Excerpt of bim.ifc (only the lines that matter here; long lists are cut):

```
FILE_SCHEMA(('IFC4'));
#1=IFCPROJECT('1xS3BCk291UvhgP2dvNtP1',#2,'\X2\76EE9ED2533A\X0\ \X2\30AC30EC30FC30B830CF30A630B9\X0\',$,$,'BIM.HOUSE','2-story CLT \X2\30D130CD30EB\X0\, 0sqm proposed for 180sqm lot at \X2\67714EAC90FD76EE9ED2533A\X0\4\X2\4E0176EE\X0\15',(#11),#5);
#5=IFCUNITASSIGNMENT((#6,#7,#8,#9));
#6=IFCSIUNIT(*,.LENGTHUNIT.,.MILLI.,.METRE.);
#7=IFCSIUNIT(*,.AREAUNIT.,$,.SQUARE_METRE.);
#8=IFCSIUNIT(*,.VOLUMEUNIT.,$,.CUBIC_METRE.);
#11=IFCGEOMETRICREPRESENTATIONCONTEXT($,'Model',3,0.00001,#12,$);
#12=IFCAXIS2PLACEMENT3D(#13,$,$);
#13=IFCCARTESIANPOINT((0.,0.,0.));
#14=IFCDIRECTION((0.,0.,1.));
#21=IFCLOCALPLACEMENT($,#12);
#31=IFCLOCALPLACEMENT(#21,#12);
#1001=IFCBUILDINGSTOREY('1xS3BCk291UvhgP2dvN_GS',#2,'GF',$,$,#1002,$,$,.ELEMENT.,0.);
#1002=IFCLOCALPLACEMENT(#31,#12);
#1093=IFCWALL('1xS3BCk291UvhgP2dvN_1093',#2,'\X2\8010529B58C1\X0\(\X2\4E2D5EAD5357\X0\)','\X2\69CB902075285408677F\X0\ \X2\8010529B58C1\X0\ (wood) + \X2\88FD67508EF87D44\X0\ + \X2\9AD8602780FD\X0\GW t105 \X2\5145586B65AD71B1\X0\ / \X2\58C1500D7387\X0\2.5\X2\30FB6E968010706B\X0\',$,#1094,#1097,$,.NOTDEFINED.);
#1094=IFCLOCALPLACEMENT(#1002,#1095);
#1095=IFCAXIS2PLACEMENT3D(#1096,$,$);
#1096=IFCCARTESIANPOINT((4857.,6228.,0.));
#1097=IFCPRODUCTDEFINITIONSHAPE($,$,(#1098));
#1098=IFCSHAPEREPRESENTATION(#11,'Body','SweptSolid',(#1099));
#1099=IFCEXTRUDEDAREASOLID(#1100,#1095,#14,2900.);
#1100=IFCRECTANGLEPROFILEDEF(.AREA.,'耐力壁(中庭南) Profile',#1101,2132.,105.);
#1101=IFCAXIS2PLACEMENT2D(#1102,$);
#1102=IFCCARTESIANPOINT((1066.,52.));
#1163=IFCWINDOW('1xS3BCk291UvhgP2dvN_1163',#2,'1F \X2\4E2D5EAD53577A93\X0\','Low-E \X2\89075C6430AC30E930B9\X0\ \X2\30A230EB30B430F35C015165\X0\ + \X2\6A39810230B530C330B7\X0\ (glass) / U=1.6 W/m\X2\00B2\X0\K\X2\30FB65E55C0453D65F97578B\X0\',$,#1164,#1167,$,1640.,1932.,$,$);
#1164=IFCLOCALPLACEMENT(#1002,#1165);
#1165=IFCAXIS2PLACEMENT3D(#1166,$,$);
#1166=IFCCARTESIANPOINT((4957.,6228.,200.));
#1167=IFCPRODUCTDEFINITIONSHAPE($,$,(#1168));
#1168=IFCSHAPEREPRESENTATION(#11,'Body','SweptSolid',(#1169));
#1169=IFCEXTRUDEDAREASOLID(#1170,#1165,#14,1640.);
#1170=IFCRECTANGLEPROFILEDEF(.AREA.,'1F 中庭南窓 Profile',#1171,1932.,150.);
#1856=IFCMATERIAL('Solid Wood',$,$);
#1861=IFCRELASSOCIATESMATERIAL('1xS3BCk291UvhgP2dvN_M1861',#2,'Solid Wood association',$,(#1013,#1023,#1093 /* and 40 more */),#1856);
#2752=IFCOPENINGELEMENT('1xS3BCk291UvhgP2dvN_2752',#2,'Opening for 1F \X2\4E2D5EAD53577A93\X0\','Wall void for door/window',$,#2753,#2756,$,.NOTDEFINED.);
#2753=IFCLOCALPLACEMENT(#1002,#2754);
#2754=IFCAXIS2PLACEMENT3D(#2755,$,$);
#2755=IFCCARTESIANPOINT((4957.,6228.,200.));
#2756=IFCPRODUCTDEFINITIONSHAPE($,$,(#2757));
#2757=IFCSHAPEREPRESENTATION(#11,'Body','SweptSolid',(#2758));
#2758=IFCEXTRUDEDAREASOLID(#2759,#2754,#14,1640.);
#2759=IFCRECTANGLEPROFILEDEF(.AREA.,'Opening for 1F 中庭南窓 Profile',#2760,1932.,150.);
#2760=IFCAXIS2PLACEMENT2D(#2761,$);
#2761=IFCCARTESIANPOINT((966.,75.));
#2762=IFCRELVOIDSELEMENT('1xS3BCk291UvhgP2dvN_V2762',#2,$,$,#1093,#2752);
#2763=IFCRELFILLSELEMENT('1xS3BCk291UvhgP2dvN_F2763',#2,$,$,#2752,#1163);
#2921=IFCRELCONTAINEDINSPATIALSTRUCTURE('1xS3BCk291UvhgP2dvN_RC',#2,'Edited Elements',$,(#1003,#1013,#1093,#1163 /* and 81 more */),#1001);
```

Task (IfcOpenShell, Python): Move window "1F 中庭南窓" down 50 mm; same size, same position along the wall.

```python
import numpy as np
import ifcopenshell
import ifcopenshell.api.geometry
import ifcopenshell.util.placement
import ifcopenshell.util.unit

model = ifcopenshell.open("bim.ifc")
unit_scale = ifcopenshell.util.unit.calculate_unit_scale(model)

window = model.by_guid("1xS3BCk291UvhgP2dvN_1163")
opening = window.FillsVoids[0].RelatingOpeningElement
dz = -0.05 / unit_scale

shift = np.array([0.0, 0.0, dz])
# The window is not placed relative to its opening, so move both.
for product in (opening, window):
    matrix = ifcopenshell.util.placement.get_local_placement(product.ObjectPlacement)
    matrix[:3, 3] += shift
    ifcopenshell.api.geometry.edit_object_placement(model, product=product, matrix=matrix, is_si=False)

print(f"moved by {dz * unit_scale:+.3f} m")

model.write("bim_v2.ifc")
```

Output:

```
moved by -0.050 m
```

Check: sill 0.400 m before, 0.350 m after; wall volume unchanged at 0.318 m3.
